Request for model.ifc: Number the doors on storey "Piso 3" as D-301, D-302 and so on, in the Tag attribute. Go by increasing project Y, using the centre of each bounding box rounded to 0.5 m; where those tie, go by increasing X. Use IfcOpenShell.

First a look at what the model holds.

```python
import ifcopenshell
import ifcopenshell.util.element
import ifcopenshell.util.placement

model = ifcopenshell.open("model.ifc")
print(model.schema)
storey = next(s for s in model.by_type("IfcBuildingStorey") if s.Name == "Piso 3")
doors = [e for e in ifcopenshell.util.element.get_decomposition(storey) if e.is_a("IfcDoor")]
for e in sorted(doors, key=lambda e: e.id()):
    origin = ifcopenshell.util.placement.get_local_placement(e.ObjectPlacement)[:3, 3]
    print(e.id(), e.Tag, e.Name, origin.round(2) + 0.0, sep=" | ")
```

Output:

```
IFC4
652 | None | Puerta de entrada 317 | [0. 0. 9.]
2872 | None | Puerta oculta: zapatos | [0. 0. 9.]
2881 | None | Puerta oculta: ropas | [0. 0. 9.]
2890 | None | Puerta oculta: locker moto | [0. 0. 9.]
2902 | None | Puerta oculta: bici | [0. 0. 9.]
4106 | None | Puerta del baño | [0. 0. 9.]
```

```python
import ifcopenshell
import ifcopenshell.geom
import ifcopenshell.util.element
import ifcopenshell.util.shape

model = ifcopenshell.open("model.ifc")
settings = ifcopenshell.geom.settings()
settings.set("use-world-coords", True)


def centre(element):
    shape = ifcopenshell.geom.create_shape(settings, element)
    return ifcopenshell.util.shape.get_bbox_centroid(shape.geometry)


storey = next(s for s in model.by_type("IfcBuildingStorey") if s.Name == "Piso 3")
doors = [e for e in ifcopenshell.util.element.get_decomposition(storey) if e.is_a("IfcDoor")]

# Insertion points can sit at a corner or the storey origin, so sort by the geometry (in metres).
centres = {e: centre(e) for e in doors}
doors.sort(key=lambda e: (round(centres[e][1] / 0.5), centres[e][0]))

for i, e in enumerate(doors, start=1):
    number = f"D-3{i:02d}"
    e.Tag = number
    print(e.id(), number)

model.write("model_updated.ifc")
```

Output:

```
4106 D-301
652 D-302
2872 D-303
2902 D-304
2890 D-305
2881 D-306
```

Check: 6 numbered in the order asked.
